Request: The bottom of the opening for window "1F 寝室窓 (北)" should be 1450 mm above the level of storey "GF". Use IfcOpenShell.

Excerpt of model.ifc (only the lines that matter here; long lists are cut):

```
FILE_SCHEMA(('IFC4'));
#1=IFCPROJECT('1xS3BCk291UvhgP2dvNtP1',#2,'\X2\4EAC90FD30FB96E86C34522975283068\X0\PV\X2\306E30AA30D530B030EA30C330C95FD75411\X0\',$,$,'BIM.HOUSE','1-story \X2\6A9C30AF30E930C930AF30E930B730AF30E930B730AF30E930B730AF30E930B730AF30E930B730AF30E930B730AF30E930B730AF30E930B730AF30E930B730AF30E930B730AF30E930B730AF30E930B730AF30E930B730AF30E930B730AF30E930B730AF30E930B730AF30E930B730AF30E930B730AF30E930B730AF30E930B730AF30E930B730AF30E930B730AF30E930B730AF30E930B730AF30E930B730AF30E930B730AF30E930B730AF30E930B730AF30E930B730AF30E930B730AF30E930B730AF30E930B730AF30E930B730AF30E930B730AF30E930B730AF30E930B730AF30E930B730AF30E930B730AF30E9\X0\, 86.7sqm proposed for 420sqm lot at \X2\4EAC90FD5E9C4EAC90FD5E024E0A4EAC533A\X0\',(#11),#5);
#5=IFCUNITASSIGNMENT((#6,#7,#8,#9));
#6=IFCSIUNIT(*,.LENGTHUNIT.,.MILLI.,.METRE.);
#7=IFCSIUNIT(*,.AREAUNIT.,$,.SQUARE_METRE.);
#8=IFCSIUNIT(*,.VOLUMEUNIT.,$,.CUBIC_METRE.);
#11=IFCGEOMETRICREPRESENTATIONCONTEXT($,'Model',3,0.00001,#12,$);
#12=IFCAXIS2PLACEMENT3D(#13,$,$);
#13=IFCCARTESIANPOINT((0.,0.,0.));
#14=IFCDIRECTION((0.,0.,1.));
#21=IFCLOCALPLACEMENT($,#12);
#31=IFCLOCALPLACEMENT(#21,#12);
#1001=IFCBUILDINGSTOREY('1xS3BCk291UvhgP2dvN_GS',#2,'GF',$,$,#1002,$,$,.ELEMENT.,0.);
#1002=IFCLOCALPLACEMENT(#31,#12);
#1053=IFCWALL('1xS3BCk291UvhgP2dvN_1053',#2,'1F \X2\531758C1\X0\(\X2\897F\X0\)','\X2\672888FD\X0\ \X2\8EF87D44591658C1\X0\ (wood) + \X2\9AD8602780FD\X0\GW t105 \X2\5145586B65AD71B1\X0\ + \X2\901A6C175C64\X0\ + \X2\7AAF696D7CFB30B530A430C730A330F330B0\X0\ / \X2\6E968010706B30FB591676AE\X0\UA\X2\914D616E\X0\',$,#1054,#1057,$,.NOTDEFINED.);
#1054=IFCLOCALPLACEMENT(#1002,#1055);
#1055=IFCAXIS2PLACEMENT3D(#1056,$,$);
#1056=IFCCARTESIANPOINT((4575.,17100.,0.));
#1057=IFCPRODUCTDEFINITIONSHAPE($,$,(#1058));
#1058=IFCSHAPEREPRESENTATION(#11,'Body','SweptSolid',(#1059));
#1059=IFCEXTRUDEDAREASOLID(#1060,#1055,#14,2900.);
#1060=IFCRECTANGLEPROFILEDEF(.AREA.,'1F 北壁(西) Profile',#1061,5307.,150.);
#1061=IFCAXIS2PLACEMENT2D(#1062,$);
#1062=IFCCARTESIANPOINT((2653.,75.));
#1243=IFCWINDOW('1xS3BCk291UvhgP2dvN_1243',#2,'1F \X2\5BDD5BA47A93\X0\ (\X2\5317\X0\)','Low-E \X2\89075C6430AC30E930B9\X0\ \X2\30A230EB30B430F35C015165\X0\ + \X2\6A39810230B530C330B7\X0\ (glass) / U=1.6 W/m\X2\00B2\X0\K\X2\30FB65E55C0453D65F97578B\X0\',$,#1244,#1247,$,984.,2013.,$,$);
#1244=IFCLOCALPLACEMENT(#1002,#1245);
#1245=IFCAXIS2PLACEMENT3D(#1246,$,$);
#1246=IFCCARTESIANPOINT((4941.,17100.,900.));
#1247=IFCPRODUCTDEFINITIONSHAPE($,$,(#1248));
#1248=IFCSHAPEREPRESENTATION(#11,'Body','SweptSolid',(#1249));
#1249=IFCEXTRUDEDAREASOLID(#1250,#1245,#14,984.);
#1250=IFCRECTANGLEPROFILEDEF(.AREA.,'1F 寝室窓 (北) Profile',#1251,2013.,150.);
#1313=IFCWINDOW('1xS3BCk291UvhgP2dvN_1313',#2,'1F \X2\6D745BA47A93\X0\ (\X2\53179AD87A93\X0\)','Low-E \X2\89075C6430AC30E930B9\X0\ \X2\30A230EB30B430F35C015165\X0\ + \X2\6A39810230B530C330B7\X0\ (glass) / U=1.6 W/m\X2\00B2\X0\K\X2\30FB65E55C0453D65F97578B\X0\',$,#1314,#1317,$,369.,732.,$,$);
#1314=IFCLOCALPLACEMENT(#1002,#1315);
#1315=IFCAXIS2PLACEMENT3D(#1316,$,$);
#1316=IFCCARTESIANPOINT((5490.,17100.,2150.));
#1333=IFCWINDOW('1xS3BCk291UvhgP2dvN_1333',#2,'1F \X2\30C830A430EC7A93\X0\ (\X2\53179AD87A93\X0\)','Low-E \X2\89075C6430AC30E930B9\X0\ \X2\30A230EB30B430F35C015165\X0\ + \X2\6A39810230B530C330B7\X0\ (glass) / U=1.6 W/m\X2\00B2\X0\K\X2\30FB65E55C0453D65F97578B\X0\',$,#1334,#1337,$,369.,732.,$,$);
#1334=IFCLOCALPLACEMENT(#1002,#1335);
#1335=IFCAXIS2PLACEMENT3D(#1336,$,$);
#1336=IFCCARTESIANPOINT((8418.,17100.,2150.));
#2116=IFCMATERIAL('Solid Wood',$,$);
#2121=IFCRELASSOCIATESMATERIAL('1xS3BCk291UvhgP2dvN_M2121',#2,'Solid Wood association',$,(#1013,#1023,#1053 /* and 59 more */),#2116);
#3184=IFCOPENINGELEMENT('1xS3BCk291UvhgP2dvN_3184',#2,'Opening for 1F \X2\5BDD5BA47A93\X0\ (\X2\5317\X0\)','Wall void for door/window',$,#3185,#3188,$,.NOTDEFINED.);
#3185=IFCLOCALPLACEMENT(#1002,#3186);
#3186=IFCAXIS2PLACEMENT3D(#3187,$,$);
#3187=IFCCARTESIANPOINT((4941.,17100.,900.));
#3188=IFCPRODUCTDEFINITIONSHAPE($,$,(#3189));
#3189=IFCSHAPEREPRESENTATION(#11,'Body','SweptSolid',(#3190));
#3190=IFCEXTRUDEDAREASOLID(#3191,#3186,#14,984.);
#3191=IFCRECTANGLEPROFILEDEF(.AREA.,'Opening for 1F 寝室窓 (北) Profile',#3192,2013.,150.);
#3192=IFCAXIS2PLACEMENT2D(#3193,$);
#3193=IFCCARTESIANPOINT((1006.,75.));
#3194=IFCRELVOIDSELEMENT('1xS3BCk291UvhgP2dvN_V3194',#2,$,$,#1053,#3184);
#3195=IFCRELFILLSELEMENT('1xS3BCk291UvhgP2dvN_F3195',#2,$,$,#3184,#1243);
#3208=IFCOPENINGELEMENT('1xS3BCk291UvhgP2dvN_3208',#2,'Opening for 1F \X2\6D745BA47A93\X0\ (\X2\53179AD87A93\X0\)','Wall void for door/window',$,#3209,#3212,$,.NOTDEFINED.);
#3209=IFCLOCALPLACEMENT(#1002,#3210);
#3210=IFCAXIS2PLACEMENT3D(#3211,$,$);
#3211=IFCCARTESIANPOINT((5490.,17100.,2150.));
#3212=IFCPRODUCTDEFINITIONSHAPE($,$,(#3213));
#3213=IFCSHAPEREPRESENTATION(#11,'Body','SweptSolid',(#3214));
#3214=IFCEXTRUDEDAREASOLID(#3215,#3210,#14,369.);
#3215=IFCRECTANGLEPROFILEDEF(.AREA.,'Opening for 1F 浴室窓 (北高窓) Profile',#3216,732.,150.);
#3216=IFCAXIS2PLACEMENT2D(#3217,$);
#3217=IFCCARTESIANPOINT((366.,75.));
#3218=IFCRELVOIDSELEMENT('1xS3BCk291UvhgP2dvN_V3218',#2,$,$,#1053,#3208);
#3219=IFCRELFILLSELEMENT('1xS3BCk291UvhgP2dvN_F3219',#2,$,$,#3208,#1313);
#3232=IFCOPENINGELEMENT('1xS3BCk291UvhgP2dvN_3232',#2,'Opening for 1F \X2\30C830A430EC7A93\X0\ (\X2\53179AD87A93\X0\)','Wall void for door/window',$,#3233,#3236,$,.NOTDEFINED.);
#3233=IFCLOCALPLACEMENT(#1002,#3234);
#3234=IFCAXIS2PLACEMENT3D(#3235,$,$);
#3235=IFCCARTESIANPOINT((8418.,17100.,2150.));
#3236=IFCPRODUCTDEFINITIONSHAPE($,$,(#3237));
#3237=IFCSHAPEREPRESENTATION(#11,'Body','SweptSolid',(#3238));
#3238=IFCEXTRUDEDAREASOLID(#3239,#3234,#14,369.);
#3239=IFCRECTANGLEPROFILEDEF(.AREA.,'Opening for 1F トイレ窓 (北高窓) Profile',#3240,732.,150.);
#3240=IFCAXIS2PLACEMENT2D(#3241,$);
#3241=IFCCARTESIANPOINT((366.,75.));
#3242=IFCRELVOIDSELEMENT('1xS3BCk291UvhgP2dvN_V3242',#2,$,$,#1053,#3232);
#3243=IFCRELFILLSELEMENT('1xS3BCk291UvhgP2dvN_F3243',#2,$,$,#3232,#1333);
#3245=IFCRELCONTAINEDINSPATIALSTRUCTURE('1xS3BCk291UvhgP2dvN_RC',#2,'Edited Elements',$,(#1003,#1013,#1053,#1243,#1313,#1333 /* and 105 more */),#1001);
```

```python
import numpy as np
import ifcopenshell
import ifcopenshell.api.geometry
import ifcopenshell.geom
import ifcopenshell.util.element
import ifcopenshell.util.placement
import ifcopenshell.util.shape
import ifcopenshell.util.unit

model = ifcopenshell.open("model.ifc")
unit_scale = ifcopenshell.util.unit.calculate_unit_scale(model)

window = model.by_id(1243)
opening = window.FillsVoids[0].RelatingOpeningElement
storey = ifcopenshell.util.element.get_container(window, ifc_class="IfcBuildingStorey")
level = ifcopenshell.util.placement.get_local_placement(storey.ObjectPlacement)[2, 3]

# The opening's origin need not be at the sill, so measure its lowest point.
shape = ifcopenshell.geom.create_shape(ifcopenshell.geom.settings(), opening)
bottom = ifcopenshell.util.shape.get_shape_bottom_elevation(shape, shape.geometry) / unit_scale
dz = level + 1.45 / unit_scale - bottom

shift = np.array([0.0, 0.0, dz])
# The window is not placed relative to its opening, so move both.
for product in (opening, window):
    matrix = ifcopenshell.util.placement.get_local_placement(product.ObjectPlacement)
    matrix[:3, 3] += shift
    ifcopenshell.api.geometry.edit_object_placement(model, product=product, matrix=matrix, is_si=False)

print(f"moved by {dz * unit_scale:+.3f} m")

model.write("model_edited.ifc")
```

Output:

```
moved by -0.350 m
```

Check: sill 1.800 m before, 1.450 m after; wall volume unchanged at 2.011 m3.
